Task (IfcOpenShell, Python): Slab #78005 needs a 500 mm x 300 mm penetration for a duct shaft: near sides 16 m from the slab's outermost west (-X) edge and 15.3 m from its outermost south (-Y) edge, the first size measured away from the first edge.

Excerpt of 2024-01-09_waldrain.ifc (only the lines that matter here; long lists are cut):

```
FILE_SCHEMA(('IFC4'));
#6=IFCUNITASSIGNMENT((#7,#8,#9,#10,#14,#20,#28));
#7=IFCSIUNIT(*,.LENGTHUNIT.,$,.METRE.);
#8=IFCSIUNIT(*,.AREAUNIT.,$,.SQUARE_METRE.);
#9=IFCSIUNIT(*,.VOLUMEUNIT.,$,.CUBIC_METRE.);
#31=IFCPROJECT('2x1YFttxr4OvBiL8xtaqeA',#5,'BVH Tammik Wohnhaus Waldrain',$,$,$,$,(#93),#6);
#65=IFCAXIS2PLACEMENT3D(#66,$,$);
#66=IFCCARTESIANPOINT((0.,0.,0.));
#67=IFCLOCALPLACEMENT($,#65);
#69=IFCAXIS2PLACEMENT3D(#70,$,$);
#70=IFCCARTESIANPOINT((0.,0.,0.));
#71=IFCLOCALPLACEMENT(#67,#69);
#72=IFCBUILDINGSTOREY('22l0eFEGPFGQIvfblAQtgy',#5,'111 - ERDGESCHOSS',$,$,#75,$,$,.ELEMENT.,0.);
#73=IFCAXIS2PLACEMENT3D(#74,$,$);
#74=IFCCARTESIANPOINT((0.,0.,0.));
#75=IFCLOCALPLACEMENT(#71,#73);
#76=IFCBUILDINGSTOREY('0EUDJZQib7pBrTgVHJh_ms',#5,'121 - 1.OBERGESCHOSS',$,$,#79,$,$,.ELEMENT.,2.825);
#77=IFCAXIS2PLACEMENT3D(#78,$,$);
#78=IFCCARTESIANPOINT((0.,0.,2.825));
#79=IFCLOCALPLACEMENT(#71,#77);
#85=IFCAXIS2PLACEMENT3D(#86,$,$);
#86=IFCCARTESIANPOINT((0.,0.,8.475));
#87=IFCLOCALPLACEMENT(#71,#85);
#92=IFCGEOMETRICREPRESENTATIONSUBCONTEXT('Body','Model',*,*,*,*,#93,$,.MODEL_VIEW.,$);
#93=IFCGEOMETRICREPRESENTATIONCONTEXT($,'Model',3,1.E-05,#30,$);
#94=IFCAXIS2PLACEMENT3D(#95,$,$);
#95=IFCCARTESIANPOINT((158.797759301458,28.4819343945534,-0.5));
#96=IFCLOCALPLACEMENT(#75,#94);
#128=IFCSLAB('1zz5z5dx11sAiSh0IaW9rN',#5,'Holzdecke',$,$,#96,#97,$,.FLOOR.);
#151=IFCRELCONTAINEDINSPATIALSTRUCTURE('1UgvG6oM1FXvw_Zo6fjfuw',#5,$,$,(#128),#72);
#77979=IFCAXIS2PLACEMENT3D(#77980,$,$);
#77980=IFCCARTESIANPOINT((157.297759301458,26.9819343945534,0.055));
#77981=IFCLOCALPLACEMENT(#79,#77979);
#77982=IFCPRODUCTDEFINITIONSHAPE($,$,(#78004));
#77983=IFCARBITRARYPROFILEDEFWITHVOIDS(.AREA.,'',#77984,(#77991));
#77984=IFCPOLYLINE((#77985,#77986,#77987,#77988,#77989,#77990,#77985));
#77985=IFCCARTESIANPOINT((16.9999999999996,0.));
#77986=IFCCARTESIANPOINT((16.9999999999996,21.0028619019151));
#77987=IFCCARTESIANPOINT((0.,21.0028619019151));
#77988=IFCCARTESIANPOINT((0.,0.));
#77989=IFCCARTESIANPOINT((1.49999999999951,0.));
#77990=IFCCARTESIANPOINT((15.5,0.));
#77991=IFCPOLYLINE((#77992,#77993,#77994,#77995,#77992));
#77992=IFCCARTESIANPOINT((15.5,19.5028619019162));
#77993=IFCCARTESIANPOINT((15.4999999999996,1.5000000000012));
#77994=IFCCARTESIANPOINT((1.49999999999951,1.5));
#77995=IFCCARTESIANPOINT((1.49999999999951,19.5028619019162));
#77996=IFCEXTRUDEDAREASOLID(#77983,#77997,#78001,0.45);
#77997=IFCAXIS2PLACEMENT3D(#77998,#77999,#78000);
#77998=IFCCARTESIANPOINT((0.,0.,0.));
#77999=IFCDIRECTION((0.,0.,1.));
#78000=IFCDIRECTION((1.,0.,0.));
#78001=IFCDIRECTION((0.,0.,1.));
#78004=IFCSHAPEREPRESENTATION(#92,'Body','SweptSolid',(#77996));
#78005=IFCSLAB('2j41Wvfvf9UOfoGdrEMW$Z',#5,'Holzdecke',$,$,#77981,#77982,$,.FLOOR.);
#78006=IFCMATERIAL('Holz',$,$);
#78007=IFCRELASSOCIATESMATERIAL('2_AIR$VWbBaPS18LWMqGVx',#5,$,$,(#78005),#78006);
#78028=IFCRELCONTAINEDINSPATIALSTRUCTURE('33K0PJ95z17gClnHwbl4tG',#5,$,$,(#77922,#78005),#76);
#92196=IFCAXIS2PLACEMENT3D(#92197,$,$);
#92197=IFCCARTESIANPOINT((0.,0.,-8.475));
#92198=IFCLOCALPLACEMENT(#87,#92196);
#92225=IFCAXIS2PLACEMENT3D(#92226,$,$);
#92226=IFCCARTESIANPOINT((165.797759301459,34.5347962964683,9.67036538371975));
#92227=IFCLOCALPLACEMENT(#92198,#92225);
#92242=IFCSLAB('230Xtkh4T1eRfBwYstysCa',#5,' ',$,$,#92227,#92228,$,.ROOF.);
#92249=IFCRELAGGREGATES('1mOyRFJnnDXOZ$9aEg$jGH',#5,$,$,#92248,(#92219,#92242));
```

```python
import numpy as np
import ifcopenshell
import ifcopenshell.api.feature
import ifcopenshell.api.geometry
import ifcopenshell.api.root
import ifcopenshell.geom
import ifcopenshell.util.placement
import ifcopenshell.util.representation
import ifcopenshell.util.shape
import ifcopenshell.util.unit

model = ifcopenshell.open("2024-01-09_waldrain.ifc")
unit_scale = ifcopenshell.util.unit.calculate_unit_scale(model)
settings = ifcopenshell.geom.settings()


def volume(element):
    """Net volume in cubic metres, openings subtracted."""
    shape = ifcopenshell.geom.create_shape(settings, element)
    return ifcopenshell.util.shape.get_volume(shape.geometry)


slab = model.by_id(78005)
before = volume(slab)

# Extent in the slab's own axes, in metres. The edges named are its -X and -Y sides.
slab_shape = ifcopenshell.geom.create_shape(settings, slab)
vertices = ifcopenshell.util.shape.get_vertices(slab_shape.geometry)
x_min, y_min, bottom = vertices.min(axis=0)
top = vertices[:, 2].max()

opening = ifcopenshell.api.root.create_entity(model, ifc_class="IfcOpeningElement", name="Duct shaft opening", predefined_type="OPENING")
context = ifcopenshell.util.representation.get_context(model, "Model", "Body", "MODEL_VIEW")
width, depth = 0.5, 0.3
outline = [(0.0, 0.0), (width, 0.0), (width, depth), (0.0, depth), (0.0, 0.0)]
# Overshoot both faces by 50 mm so the cut is clean.
shape = ifcopenshell.api.geometry.add_slab_representation(
    model, context=context, depth=top - bottom + 0.1, polyline=outline
)
ifcopenshell.api.geometry.assign_representation(model, product=opening, representation=shape)

matrix = ifcopenshell.util.placement.get_local_placement(slab.ObjectPlacement)
matrix[:, 3] = matrix @ np.append(np.array([x_min + 16, y_min + 15.3, bottom - 0.05]) / unit_scale, 1.0)
ifcopenshell.api.geometry.edit_object_placement(model, product=opening, matrix=matrix, is_si=False)
ifcopenshell.api.feature.add_feature(model, feature=opening, element=slab)

after = volume(slab)

print(f"slab volume {before:.3f} -> {after:.3f} m3")

model.write("2024-01-09_waldrain_edited.ifc")
```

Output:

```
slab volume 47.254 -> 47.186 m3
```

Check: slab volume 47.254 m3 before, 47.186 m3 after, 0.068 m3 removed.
